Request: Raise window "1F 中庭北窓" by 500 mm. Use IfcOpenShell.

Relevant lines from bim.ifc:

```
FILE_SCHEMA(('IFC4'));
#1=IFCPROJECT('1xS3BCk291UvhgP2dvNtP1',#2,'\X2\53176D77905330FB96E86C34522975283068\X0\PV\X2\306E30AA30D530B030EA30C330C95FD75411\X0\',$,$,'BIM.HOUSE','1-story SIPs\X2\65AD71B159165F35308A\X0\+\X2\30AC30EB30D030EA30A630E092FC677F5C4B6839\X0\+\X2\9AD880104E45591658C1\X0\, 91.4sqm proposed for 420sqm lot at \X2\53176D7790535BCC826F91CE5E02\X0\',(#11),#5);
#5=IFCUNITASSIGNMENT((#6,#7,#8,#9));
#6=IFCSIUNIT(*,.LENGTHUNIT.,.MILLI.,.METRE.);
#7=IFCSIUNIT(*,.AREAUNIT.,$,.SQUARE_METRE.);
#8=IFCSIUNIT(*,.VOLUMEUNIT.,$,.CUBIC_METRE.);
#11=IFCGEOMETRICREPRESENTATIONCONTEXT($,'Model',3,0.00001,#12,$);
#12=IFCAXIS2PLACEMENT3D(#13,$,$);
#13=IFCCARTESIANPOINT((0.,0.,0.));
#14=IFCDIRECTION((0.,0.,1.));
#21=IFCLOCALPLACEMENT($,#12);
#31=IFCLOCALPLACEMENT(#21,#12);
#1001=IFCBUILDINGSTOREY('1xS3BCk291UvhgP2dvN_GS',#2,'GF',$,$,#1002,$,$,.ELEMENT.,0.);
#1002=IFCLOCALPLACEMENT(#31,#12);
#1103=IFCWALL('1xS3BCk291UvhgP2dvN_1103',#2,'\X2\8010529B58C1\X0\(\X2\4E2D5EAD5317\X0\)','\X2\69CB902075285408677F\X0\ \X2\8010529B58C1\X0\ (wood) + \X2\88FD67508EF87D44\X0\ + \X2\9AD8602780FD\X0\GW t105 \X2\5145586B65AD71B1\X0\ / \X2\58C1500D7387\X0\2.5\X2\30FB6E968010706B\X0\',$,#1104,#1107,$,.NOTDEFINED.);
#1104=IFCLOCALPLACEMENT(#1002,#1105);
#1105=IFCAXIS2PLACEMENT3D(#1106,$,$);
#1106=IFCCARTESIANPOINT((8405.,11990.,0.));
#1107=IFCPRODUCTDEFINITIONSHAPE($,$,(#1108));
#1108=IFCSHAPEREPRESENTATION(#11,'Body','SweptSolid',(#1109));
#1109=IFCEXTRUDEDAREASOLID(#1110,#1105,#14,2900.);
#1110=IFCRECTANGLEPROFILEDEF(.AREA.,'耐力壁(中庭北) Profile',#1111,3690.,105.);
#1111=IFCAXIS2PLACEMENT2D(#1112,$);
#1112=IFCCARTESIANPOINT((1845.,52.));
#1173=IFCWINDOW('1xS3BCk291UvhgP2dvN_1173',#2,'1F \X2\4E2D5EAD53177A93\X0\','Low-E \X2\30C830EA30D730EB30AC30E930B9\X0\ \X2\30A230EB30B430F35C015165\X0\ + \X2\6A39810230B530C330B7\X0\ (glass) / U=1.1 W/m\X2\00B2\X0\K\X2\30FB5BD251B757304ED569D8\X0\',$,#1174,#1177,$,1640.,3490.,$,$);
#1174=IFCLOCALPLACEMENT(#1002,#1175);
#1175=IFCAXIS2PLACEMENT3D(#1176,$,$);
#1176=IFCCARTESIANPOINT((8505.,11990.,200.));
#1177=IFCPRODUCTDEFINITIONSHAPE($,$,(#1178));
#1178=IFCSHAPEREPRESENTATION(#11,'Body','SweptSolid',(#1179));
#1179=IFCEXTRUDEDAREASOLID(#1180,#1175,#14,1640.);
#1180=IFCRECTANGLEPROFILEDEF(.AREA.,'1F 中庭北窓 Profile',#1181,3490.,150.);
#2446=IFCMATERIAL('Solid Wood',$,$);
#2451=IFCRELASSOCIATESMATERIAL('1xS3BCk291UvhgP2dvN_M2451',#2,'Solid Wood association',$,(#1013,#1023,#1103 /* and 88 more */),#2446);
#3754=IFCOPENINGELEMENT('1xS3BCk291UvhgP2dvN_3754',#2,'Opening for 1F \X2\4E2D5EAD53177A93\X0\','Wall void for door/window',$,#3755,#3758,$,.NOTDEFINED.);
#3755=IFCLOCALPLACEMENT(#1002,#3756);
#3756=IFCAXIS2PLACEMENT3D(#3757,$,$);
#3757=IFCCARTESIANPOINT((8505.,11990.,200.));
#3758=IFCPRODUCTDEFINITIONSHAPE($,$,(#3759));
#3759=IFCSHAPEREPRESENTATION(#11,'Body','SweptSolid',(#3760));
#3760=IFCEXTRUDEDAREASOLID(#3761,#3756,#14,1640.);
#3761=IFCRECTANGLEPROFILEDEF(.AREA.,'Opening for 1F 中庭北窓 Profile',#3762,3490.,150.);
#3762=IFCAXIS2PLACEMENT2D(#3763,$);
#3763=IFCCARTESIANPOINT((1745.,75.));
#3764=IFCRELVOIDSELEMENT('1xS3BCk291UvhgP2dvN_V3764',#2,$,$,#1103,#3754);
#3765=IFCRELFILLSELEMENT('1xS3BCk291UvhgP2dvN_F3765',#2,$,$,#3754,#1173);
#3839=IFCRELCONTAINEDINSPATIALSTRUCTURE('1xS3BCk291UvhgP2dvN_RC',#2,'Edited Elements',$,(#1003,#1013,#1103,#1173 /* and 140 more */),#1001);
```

```python
import numpy as np
import ifcopenshell
import ifcopenshell.api.geometry
import ifcopenshell.util.placement
import ifcopenshell.util.unit

model = ifcopenshell.open("bim.ifc")
unit_scale = ifcopenshell.util.unit.calculate_unit_scale(model)

window = model.by_guid("1xS3BCk291UvhgP2dvN_1173")
opening = window.FillsVoids[0].RelatingOpeningElement
dz = 0.5 / unit_scale

shift = np.array([0.0, 0.0, dz])
# The window is not placed relative to its opening, so move both.
for product in (opening, window):
    matrix = ifcopenshell.util.placement.get_local_placement(product.ObjectPlacement)
    matrix[:3, 3] += shift
    ifcopenshell.api.geometry.edit_object_placement(model, product=product, matrix=matrix, is_si=False)

print(f"moved by {dz * unit_scale:+.3f} m")

model.write("bim_rev.ifc")
```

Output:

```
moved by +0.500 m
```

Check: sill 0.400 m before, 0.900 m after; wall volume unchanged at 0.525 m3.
